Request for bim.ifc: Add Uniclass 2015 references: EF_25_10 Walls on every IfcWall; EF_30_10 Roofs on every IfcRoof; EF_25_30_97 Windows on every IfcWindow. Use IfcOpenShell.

First a look at what the model holds.

```python
import ifcopenshell

model = ifcopenshell.open("bim.ifc")
print(model.schema)
print("classifications:", [c.Name for c in model.by_type("IfcClassification")])
for ifc_class in ("IfcDoor", "IfcRoof", "IfcStair", "IfcWall", "IfcWindow"):
    print(ifc_class, len(model.by_type(ifc_class)))
```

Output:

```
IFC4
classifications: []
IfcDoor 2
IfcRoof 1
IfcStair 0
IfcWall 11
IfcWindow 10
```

```python
import ifcopenshell
import ifcopenshell.api.classification

model = ifcopenshell.open("bim.ifc")

system = ifcopenshell.api.classification.add_classification(model, classification="Uniclass 2015")

codes = {
    "IfcWall": ("EF_25_10", "Walls"),
    "IfcRoof": ("EF_30_10", "Roofs"),
    "IfcWindow": ("EF_25_30_97", "Windows"),
}
for ifc_class, (code, name) in codes.items():
    products = model.by_type(ifc_class)
    ifcopenshell.api.classification.add_reference(
        model, products=products, classification=system, identification=code, name=name
    )
    print(code, len(products))

model.write("bim_v2.ifc")
```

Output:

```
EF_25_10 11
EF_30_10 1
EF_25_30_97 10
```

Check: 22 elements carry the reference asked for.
